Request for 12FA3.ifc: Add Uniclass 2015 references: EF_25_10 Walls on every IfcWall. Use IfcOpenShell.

First a look at what the model holds.

```python
import ifcopenshell

model = ifcopenshell.open("12FA3.ifc")
print(model.schema)
print("classifications:", [c.Name for c in model.by_type("IfcClassification")])
for ifc_class in ("IfcDoor", "IfcRoof", "IfcStair", "IfcWall", "IfcWindow"):
    print(ifc_class, len(model.by_type(ifc_class)))
```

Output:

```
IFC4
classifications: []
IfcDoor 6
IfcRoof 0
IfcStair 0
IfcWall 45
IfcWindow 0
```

```python
import ifcopenshell
import ifcopenshell.api.classification

model = ifcopenshell.open("12FA3.ifc")

system = ifcopenshell.api.classification.add_classification(model, classification="Uniclass 2015")

codes = {
    "IfcWall": ("EF_25_10", "Walls"),
}
for ifc_class, (code, name) in codes.items():
    products = model.by_type(ifc_class)
    ifcopenshell.api.classification.add_reference(
        model, products=products, classification=system, identification=code, name=name
    )
    print(code, len(products))

model.write("12FA3_updated.ifc")
```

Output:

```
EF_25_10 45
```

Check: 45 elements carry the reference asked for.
